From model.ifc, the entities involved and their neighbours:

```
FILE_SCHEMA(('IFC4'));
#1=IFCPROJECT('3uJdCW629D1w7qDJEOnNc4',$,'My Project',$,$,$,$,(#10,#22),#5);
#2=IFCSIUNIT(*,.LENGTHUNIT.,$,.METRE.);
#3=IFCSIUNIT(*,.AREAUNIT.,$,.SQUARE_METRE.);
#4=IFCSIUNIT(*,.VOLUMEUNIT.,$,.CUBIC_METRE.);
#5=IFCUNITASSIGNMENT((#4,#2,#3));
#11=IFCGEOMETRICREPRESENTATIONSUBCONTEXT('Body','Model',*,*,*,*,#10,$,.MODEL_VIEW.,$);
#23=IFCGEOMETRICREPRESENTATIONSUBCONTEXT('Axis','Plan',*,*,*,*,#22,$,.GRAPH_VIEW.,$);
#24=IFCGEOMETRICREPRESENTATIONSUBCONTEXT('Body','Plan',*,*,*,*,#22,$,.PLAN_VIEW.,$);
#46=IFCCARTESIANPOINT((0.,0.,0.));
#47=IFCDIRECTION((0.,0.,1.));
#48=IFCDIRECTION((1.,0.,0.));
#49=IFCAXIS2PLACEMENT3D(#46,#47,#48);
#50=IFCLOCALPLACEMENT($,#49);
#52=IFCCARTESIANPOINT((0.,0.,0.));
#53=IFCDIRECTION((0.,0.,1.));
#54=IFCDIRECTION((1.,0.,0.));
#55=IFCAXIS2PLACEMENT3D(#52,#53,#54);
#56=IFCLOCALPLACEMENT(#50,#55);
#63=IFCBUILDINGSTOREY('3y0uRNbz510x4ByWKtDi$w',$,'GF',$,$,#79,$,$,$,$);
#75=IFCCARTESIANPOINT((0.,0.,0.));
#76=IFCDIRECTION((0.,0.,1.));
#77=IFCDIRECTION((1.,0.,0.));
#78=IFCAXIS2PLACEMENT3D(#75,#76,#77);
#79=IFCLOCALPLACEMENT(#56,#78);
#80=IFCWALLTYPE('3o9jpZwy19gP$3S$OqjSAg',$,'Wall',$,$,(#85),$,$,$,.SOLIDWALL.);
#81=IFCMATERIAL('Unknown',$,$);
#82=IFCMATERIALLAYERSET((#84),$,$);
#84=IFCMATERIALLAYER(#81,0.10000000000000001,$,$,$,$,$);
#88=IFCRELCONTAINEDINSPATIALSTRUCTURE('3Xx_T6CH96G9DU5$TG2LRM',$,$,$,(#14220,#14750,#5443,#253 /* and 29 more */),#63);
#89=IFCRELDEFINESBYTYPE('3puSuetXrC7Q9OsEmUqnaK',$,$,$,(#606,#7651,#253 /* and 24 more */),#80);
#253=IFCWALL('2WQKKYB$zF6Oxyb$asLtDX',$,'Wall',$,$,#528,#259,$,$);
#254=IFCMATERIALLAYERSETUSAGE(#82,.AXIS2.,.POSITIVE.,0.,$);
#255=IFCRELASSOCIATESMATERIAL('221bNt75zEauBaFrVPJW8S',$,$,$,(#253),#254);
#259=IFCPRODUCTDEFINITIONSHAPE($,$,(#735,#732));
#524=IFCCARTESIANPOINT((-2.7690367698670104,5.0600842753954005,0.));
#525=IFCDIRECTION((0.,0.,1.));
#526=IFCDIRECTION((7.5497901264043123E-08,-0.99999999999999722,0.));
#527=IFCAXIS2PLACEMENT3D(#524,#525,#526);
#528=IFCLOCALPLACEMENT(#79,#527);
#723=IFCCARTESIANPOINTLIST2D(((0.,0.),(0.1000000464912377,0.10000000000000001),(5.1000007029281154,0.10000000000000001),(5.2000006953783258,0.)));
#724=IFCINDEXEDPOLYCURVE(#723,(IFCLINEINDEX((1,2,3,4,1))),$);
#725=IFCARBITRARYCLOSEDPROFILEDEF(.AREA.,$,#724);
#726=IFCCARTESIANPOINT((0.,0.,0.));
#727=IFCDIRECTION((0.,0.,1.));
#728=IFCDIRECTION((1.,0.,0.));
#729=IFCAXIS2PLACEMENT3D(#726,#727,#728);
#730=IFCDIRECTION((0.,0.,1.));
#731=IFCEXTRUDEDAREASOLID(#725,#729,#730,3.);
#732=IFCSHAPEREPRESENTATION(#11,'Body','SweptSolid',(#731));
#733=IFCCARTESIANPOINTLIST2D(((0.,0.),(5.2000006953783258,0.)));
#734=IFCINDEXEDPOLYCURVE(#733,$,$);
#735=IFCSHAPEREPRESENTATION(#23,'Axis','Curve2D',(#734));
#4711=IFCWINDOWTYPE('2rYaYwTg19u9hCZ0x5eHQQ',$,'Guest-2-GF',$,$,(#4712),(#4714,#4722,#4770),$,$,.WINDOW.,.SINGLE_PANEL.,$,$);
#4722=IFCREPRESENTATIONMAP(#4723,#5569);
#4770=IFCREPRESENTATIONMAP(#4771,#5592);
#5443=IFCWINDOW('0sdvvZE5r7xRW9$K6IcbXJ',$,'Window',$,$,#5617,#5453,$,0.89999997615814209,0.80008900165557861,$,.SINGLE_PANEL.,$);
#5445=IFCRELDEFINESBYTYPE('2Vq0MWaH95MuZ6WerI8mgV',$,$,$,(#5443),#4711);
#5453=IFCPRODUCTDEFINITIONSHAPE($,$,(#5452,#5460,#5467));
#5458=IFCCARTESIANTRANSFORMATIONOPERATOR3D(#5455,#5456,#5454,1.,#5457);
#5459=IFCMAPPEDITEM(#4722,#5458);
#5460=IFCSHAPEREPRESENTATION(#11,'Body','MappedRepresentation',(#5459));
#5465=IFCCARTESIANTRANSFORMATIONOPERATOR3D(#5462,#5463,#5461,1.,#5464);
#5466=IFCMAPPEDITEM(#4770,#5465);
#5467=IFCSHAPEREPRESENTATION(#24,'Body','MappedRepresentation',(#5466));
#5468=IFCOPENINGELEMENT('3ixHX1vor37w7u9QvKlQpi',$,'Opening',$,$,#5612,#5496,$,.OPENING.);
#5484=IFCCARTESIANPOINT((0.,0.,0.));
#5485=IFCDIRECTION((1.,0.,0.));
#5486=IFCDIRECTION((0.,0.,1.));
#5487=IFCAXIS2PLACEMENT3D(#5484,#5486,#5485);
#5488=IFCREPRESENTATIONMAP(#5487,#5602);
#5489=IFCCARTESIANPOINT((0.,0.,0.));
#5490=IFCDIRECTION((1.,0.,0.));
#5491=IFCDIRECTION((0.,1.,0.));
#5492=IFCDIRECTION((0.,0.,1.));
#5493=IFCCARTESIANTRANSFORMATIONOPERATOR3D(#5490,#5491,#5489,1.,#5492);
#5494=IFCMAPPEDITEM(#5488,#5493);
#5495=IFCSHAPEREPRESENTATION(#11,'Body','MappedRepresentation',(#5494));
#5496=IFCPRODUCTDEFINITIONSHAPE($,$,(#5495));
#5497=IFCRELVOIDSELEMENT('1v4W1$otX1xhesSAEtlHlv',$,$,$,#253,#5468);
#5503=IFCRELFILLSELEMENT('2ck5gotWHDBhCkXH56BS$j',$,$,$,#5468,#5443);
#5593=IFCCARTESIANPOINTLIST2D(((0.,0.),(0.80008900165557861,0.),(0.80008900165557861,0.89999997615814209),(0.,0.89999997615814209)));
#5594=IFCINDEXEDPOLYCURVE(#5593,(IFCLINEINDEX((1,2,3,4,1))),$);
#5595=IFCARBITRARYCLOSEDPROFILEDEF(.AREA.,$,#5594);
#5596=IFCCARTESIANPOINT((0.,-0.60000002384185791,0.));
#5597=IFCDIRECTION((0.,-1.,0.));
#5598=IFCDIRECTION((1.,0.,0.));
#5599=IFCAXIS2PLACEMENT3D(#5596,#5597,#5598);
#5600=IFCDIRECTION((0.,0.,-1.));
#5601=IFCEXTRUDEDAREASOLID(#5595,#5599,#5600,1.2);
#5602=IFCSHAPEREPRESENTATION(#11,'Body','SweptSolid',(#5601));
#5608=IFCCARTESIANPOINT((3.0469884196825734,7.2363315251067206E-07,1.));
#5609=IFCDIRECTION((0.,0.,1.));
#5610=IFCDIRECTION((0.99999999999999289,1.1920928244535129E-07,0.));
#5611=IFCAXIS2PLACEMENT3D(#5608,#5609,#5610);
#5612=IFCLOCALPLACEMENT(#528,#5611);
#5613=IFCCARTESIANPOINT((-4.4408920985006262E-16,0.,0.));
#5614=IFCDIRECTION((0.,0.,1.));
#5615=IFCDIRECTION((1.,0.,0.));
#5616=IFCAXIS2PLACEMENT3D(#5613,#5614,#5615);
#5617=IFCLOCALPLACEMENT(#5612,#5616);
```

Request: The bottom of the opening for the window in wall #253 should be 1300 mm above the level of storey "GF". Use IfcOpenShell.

```python
import numpy as np
import ifcopenshell
import ifcopenshell.api.geometry
import ifcopenshell.geom
import ifcopenshell.util.element
import ifcopenshell.util.placement
import ifcopenshell.util.shape
import ifcopenshell.util.unit

model = ifcopenshell.open("model.ifc")
unit_scale = ifcopenshell.util.unit.calculate_unit_scale(model)

window = model.by_guid("0sdvvZE5r7xRW9$K6IcbXJ")
opening = window.FillsVoids[0].RelatingOpeningElement
storey = ifcopenshell.util.element.get_container(window, ifc_class="IfcBuildingStorey")
level = ifcopenshell.util.placement.get_local_placement(storey.ObjectPlacement)[2, 3]

# The opening's origin need not be at the sill, so measure its lowest point.
shape = ifcopenshell.geom.create_shape(ifcopenshell.geom.settings(), opening)
bottom = ifcopenshell.util.shape.get_shape_bottom_elevation(shape, shape.geometry) / unit_scale
dz = level + 1.3 - bottom

shift = np.array([0.0, 0.0, dz])
# The window is placed relative to its opening, so it follows when the opening moves.
matrix = ifcopenshell.util.placement.get_local_placement(opening.ObjectPlacement)
matrix[:3, 3] += shift
ifcopenshell.api.geometry.edit_object_placement(
    model, product=opening, matrix=matrix, is_si=False, should_transform_children=True
)

print(f"moved by {dz * unit_scale:+.3f} m")

model.write("model_edited.ifc")
```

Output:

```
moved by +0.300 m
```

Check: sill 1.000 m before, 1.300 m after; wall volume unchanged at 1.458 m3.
